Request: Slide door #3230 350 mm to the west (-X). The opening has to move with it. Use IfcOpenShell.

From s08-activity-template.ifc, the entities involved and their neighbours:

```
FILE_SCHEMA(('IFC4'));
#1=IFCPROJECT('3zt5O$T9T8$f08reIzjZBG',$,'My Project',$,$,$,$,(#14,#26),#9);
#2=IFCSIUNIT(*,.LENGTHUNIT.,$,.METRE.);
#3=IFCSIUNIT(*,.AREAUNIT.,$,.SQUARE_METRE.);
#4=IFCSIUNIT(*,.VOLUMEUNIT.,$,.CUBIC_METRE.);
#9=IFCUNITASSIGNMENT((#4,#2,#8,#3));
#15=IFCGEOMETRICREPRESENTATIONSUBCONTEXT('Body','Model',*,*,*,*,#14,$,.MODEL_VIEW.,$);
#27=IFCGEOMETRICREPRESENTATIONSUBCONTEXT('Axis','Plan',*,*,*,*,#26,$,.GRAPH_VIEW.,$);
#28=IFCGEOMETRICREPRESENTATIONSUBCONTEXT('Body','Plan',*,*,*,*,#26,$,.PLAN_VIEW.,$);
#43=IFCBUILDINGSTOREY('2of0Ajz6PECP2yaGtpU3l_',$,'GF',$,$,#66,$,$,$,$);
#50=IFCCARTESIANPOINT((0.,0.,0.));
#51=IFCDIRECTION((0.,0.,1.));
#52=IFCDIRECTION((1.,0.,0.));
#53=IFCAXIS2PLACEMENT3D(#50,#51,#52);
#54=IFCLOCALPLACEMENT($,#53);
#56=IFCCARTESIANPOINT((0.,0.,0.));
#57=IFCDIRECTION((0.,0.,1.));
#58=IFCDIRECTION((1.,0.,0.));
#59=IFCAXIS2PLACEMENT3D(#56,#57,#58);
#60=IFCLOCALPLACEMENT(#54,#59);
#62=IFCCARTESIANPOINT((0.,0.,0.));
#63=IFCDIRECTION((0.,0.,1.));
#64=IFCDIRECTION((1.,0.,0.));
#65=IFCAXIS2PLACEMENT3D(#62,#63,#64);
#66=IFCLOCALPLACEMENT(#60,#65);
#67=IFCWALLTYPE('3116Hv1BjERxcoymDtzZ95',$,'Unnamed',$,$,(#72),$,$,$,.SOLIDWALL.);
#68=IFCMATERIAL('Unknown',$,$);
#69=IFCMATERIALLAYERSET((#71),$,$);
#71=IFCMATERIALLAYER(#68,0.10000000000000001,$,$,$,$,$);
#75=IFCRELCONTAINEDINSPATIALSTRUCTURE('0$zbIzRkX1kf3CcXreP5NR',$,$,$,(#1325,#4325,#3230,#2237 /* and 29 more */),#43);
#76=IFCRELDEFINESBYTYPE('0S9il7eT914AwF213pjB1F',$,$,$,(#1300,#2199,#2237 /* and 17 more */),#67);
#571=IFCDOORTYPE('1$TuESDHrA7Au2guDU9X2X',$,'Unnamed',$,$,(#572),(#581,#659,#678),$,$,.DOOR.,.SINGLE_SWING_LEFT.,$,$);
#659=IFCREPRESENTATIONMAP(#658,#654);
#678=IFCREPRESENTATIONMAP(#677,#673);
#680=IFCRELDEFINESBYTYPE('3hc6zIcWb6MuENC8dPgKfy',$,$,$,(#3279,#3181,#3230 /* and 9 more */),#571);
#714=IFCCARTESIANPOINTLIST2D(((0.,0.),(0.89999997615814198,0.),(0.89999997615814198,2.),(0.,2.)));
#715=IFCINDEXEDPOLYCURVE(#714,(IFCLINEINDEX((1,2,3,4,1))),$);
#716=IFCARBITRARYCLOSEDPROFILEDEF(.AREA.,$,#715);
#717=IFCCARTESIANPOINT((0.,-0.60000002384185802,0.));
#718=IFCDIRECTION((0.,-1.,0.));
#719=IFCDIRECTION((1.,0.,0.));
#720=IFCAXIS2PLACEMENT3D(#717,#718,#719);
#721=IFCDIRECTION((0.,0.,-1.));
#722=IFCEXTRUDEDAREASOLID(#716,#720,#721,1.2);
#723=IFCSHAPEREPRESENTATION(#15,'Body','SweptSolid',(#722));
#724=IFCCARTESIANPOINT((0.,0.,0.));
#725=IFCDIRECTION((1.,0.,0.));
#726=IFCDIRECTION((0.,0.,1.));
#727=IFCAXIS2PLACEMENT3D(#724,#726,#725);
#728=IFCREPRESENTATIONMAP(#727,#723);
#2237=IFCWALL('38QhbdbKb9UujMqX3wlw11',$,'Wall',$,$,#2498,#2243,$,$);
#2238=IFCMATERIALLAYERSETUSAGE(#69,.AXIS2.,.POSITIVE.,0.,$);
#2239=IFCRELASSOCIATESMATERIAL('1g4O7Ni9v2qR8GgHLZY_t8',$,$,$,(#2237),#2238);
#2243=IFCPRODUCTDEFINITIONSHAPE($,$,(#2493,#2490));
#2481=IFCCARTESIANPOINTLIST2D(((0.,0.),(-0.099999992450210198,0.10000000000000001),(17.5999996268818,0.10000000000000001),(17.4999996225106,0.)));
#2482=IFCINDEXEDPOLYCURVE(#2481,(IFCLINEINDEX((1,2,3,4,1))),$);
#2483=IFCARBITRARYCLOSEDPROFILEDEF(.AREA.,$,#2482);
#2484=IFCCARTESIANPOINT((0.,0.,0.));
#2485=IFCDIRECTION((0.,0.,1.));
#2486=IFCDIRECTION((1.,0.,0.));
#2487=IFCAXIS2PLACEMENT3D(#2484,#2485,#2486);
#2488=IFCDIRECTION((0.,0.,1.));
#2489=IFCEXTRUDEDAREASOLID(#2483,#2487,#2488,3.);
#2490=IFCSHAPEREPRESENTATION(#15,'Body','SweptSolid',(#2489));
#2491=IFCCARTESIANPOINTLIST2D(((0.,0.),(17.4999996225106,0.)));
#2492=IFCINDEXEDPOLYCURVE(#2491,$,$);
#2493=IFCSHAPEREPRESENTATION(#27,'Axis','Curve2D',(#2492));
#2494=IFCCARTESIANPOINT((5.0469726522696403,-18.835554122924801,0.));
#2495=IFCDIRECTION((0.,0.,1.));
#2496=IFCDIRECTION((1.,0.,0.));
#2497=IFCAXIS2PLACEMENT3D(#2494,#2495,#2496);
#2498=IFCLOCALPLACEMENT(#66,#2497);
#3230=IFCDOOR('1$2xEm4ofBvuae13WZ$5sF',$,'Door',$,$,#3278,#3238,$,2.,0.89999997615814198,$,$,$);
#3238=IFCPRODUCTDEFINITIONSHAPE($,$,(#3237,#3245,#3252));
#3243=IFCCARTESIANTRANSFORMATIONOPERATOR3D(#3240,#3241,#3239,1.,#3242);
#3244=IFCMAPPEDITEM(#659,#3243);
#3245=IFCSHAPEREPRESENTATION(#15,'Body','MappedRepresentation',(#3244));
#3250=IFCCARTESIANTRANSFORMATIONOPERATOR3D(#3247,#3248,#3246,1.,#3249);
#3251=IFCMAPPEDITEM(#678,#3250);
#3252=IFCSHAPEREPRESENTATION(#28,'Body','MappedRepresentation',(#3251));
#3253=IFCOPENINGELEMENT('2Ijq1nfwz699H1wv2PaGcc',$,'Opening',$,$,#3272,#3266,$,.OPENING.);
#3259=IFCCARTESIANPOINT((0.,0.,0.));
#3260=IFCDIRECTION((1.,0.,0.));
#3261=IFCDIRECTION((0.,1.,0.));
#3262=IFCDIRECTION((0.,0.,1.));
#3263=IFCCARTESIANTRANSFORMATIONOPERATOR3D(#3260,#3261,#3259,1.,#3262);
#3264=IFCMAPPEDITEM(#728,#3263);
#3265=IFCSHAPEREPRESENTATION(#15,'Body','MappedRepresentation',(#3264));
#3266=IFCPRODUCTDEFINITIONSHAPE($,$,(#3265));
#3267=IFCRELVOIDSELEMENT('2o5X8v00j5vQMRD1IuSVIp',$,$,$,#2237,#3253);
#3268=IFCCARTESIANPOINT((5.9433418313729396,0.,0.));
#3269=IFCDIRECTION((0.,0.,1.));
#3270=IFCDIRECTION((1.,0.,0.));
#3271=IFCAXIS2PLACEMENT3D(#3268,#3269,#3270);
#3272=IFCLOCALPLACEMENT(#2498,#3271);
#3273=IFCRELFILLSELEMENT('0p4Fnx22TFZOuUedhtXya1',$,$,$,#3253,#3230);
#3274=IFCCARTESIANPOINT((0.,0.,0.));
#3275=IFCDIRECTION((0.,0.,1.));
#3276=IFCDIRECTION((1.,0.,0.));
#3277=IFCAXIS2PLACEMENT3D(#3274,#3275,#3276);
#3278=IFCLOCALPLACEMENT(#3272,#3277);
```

```python
import ifcopenshell
import ifcopenshell.api.geometry
import ifcopenshell.util.placement

model = ifcopenshell.open("s08-activity-template.ifc")

door = model.by_guid("1$2xEm4ofBvuae13WZ$5sF")
opening = door.FillsVoids[0].RelatingOpeningElement
wall = opening.VoidsElements[0].RelatingBuildingElement

wall_matrix = ifcopenshell.util.placement.get_local_placement(wall.ObjectPlacement)
shift = wall_matrix[:3, 0] * -0.35
before = ifcopenshell.util.placement.get_local_placement(door.ObjectPlacement)[:3, 3].copy()

# The door is placed relative to its opening, so it follows when the opening moves.
matrix = ifcopenshell.util.placement.get_local_placement(opening.ObjectPlacement)
matrix[:3, 3] += shift
ifcopenshell.api.geometry.edit_object_placement(
    model, product=opening, matrix=matrix, is_si=False, should_transform_children=True
)

after = ifcopenshell.util.placement.get_local_placement(door.ObjectPlacement)[:3, 3]
print("door moved by", (after - before).round(3) + 0.0)

model.write("s08-activity-template-out.ifc")
```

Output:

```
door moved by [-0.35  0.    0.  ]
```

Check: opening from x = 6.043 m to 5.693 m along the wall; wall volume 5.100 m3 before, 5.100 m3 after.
